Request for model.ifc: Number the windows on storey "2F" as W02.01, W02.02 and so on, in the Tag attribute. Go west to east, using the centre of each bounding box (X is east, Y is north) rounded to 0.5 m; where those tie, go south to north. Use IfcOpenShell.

First a look at what the model holds.

```python
import ifcopenshell
import ifcopenshell.util.element
import ifcopenshell.util.placement

model = ifcopenshell.open("model.ifc")
print(model.schema)
storey = next(s for s in model.by_type("IfcBuildingStorey") if s.Name == "2F")
windows = [e for e in ifcopenshell.util.element.get_decomposition(storey) if e.is_a("IfcWindow")]
for e in sorted(windows, key=lambda e: e.id()):
    origin = ifcopenshell.util.placement.get_local_placement(e.ObjectPlacement)[:3, 3]
    print(e.id(), e.Tag, e.Name, origin.round(2) + 0.0, sep=" | ")
```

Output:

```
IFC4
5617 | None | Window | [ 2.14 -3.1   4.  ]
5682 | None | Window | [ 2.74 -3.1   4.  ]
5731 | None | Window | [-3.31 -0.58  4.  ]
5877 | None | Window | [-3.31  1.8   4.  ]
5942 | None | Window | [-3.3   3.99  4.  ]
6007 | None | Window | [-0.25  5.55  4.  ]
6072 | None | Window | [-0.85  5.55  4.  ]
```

```python
import ifcopenshell
import ifcopenshell.geom
import ifcopenshell.util.element
import ifcopenshell.util.shape

model = ifcopenshell.open("model.ifc")
settings = ifcopenshell.geom.settings()
settings.set("use-world-coords", True)


def centre(element):
    shape = ifcopenshell.geom.create_shape(settings, element)
    return ifcopenshell.util.shape.get_bbox_centroid(shape.geometry)


storey = next(s for s in model.by_type("IfcBuildingStorey") if s.Name == "2F")
windows = [e for e in ifcopenshell.util.element.get_decomposition(storey) if e.is_a("IfcWindow")]

# Insertion points can sit at a corner or the storey origin, so sort by the geometry (in metres).
centres = {e: centre(e) for e in windows}
windows.sort(key=lambda e: (round(centres[e][0] / 0.5), centres[e][1]))

for i, e in enumerate(windows, start=1):
    number = f"W02.{i:02d}"
    e.Tag = number
    print(e.id(), number)

model.write("model_updated.ifc")
```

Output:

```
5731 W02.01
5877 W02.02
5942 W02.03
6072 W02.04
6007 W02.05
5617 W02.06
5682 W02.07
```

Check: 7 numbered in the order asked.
